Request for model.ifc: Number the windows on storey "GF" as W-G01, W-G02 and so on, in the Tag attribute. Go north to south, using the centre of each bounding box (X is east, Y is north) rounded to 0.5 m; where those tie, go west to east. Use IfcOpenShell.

First a look at what the model holds.

```python
import ifcopenshell
import ifcopenshell.util.element
import ifcopenshell.util.placement

model = ifcopenshell.open("model.ifc")
print(model.schema)
storey = next(s for s in model.by_type("IfcBuildingStorey") if s.Name == "GF")
windows = [e for e in ifcopenshell.util.element.get_decomposition(storey) if e.is_a("IfcWindow")]
for e in sorted(windows, key=lambda e: e.id()):
    origin = ifcopenshell.util.placement.get_local_placement(e.ObjectPlacement)[:3, 3]
    print(e.id(), e.Tag, e.Name, origin.round(2) + 0.0, sep=" | ")
```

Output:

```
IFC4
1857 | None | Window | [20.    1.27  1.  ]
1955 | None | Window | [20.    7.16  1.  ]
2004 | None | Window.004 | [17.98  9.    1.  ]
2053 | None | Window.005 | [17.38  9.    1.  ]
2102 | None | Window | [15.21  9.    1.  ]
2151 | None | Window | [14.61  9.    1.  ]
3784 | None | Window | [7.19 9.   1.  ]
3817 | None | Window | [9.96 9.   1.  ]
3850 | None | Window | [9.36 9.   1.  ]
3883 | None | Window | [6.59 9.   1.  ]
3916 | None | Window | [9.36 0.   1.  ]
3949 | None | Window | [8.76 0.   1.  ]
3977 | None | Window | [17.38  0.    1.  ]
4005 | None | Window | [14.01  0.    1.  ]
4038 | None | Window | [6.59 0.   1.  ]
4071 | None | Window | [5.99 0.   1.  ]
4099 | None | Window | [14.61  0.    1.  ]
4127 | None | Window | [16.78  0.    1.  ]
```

```python
import ifcopenshell
import ifcopenshell.geom
import ifcopenshell.util.element
import ifcopenshell.util.shape

model = ifcopenshell.open("model.ifc")
settings = ifcopenshell.geom.settings()
settings.set("use-world-coords", True)


def centre(element):
    shape = ifcopenshell.geom.create_shape(settings, element)
    return ifcopenshell.util.shape.get_bbox_centroid(shape.geometry)


storey = next(s for s in model.by_type("IfcBuildingStorey") if s.Name == "GF")
windows = [e for e in ifcopenshell.util.element.get_decomposition(storey) if e.is_a("IfcWindow")]

# Insertion points can sit at a corner or the storey origin, so sort by the geometry (in metres).
centres = {e: centre(e) for e in windows}
windows.sort(key=lambda e: (-round(centres[e][1] / 0.5), centres[e][0]))

for i, e in enumerate(windows, start=1):
    number = f"W-G{i:02d}"
    e.Tag = number
    print(e.id(), number)

model.write("model_updated.ifc")
```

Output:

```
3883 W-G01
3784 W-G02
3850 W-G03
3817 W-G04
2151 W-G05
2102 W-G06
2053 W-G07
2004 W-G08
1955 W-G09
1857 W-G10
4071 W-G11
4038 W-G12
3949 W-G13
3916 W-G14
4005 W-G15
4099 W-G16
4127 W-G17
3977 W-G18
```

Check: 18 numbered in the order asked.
